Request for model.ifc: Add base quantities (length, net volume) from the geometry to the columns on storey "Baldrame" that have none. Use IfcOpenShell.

First a look at what the model holds.

```python
import ifcopenshell
import ifcopenshell.util.element
import ifcopenshell.util.unit

model = ifcopenshell.open("model.ifc")
print(model.schema)
for unit_type in ("LENGTHUNIT", "AREAUNIT", "VOLUMEUNIT"):
    print(unit_type, ifcopenshell.util.unit.calculate_unit_scale(model, unit_type))
storey = next(s for s in model.by_type("IfcBuildingStorey") if s.Name == "Baldrame")
columns = [e for e in ifcopenshell.util.element.get_decomposition(storey) if e.is_a("IfcColumn")]
for e in sorted(columns, key=lambda e: e.id()):
    print(e.id(), e.is_a(), e.Name, list(ifcopenshell.util.element.get_psets(e, qtos_only=True)), sep=" | ")
```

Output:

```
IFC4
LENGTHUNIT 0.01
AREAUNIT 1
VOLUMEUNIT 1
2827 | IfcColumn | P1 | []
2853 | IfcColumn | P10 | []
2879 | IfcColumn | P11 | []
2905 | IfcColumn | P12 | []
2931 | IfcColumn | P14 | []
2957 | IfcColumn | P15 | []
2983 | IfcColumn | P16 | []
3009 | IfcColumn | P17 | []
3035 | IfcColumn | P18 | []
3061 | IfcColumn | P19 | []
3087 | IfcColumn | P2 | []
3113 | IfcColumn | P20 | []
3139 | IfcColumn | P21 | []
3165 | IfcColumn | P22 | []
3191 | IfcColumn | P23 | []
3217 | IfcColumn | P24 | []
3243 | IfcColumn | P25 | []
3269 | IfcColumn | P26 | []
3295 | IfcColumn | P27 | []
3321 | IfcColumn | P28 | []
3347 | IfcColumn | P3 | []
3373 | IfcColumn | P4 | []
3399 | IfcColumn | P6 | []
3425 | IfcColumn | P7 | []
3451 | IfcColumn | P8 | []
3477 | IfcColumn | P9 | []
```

```python
import ifcopenshell
import ifcopenshell.api.pset
import ifcopenshell.geom
import ifcopenshell.util.element
import ifcopenshell.util.shape
import ifcopenshell.util.unit

model = ifcopenshell.open("model.ifc")
unit_scale = ifcopenshell.util.unit.calculate_unit_scale(model)
volume_scale = ifcopenshell.util.unit.calculate_unit_scale(model, "VOLUMEUNIT")
settings = ifcopenshell.geom.settings()

storey = next(s for s in model.by_type("IfcBuildingStorey") if s.Name == "Baldrame")
columns = [e for e in ifcopenshell.util.element.get_decomposition(storey) if e.is_a("IfcColumn")]

for e in sorted(columns, key=lambda e: e.id()):
    if ifcopenshell.util.element.get_psets(e, qtos_only=True, should_inherit=False):
        continue
    # Geometry comes back in metres, in the element's own axes.
    shape = ifcopenshell.geom.create_shape(settings, e)
    values = {
        "Length": ifcopenshell.util.shape.get_z(shape.geometry) / unit_scale,
        "NetVolume": ifcopenshell.util.shape.get_volume(shape.geometry) / volume_scale,
    }
    qto = ifcopenshell.api.pset.add_qto(model, product=e, name="Qto_ColumnBaseQuantities")
    ifcopenshell.api.pset.edit_qto(model, qto=qto, properties=values)
    print(e.id(), {k: round(v, 3) for k, v in values.items()})

model.write("model_rev.ifc")
```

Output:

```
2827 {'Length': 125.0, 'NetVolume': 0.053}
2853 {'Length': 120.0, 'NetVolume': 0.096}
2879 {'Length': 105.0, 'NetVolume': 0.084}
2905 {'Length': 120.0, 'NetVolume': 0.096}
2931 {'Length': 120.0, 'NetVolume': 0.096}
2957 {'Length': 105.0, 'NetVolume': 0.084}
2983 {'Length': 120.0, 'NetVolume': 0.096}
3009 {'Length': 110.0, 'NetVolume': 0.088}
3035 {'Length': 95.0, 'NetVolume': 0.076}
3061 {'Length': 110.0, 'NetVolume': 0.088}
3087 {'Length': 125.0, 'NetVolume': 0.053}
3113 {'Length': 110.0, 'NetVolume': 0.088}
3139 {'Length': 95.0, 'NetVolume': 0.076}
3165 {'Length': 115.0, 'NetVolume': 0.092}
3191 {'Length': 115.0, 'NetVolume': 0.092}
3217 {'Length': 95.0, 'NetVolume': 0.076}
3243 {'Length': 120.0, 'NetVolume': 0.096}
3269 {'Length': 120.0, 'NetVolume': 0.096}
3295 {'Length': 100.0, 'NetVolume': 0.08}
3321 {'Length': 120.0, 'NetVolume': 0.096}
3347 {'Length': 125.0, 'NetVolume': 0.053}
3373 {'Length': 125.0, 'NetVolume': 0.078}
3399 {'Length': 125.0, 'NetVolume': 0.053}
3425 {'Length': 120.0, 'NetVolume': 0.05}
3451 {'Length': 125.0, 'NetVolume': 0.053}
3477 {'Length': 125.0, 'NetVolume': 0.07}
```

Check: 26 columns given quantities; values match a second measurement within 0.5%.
